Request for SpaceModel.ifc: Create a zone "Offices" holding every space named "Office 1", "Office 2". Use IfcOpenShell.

First a look at what the model holds.

```python
import ifcopenshell

model = ifcopenshell.open("SpaceModel.ifc")
print(model.schema)
seen = {}
for space in model.by_type("IfcSpace"):
    seen[space.LongName] = seen.get(space.LongName, 0) + 1
for name, count in sorted(seen.items(), key=str):
    print(count, "x", name)
print("zones:", [z.Name for z in model.by_type("IfcZone")][:20])
```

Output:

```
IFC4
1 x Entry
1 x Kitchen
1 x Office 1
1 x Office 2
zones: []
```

```python
import ifcopenshell
import ifcopenshell.api.group
import ifcopenshell.api.root

model = ifcopenshell.open("SpaceModel.ifc")

names = {"Office 1", "Office 2"}
spaces = [s for s in model.by_type("IfcSpace") if s.LongName in names]

zone = ifcopenshell.api.root.create_entity(model, ifc_class="IfcZone", name="Offices")
ifcopenshell.api.group.assign_group(model, products=spaces, group=zone)
print(len(spaces), "spaces in", zone.Name)

model.write("SpaceModel_v2.ifc")
```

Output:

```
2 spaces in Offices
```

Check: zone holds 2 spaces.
